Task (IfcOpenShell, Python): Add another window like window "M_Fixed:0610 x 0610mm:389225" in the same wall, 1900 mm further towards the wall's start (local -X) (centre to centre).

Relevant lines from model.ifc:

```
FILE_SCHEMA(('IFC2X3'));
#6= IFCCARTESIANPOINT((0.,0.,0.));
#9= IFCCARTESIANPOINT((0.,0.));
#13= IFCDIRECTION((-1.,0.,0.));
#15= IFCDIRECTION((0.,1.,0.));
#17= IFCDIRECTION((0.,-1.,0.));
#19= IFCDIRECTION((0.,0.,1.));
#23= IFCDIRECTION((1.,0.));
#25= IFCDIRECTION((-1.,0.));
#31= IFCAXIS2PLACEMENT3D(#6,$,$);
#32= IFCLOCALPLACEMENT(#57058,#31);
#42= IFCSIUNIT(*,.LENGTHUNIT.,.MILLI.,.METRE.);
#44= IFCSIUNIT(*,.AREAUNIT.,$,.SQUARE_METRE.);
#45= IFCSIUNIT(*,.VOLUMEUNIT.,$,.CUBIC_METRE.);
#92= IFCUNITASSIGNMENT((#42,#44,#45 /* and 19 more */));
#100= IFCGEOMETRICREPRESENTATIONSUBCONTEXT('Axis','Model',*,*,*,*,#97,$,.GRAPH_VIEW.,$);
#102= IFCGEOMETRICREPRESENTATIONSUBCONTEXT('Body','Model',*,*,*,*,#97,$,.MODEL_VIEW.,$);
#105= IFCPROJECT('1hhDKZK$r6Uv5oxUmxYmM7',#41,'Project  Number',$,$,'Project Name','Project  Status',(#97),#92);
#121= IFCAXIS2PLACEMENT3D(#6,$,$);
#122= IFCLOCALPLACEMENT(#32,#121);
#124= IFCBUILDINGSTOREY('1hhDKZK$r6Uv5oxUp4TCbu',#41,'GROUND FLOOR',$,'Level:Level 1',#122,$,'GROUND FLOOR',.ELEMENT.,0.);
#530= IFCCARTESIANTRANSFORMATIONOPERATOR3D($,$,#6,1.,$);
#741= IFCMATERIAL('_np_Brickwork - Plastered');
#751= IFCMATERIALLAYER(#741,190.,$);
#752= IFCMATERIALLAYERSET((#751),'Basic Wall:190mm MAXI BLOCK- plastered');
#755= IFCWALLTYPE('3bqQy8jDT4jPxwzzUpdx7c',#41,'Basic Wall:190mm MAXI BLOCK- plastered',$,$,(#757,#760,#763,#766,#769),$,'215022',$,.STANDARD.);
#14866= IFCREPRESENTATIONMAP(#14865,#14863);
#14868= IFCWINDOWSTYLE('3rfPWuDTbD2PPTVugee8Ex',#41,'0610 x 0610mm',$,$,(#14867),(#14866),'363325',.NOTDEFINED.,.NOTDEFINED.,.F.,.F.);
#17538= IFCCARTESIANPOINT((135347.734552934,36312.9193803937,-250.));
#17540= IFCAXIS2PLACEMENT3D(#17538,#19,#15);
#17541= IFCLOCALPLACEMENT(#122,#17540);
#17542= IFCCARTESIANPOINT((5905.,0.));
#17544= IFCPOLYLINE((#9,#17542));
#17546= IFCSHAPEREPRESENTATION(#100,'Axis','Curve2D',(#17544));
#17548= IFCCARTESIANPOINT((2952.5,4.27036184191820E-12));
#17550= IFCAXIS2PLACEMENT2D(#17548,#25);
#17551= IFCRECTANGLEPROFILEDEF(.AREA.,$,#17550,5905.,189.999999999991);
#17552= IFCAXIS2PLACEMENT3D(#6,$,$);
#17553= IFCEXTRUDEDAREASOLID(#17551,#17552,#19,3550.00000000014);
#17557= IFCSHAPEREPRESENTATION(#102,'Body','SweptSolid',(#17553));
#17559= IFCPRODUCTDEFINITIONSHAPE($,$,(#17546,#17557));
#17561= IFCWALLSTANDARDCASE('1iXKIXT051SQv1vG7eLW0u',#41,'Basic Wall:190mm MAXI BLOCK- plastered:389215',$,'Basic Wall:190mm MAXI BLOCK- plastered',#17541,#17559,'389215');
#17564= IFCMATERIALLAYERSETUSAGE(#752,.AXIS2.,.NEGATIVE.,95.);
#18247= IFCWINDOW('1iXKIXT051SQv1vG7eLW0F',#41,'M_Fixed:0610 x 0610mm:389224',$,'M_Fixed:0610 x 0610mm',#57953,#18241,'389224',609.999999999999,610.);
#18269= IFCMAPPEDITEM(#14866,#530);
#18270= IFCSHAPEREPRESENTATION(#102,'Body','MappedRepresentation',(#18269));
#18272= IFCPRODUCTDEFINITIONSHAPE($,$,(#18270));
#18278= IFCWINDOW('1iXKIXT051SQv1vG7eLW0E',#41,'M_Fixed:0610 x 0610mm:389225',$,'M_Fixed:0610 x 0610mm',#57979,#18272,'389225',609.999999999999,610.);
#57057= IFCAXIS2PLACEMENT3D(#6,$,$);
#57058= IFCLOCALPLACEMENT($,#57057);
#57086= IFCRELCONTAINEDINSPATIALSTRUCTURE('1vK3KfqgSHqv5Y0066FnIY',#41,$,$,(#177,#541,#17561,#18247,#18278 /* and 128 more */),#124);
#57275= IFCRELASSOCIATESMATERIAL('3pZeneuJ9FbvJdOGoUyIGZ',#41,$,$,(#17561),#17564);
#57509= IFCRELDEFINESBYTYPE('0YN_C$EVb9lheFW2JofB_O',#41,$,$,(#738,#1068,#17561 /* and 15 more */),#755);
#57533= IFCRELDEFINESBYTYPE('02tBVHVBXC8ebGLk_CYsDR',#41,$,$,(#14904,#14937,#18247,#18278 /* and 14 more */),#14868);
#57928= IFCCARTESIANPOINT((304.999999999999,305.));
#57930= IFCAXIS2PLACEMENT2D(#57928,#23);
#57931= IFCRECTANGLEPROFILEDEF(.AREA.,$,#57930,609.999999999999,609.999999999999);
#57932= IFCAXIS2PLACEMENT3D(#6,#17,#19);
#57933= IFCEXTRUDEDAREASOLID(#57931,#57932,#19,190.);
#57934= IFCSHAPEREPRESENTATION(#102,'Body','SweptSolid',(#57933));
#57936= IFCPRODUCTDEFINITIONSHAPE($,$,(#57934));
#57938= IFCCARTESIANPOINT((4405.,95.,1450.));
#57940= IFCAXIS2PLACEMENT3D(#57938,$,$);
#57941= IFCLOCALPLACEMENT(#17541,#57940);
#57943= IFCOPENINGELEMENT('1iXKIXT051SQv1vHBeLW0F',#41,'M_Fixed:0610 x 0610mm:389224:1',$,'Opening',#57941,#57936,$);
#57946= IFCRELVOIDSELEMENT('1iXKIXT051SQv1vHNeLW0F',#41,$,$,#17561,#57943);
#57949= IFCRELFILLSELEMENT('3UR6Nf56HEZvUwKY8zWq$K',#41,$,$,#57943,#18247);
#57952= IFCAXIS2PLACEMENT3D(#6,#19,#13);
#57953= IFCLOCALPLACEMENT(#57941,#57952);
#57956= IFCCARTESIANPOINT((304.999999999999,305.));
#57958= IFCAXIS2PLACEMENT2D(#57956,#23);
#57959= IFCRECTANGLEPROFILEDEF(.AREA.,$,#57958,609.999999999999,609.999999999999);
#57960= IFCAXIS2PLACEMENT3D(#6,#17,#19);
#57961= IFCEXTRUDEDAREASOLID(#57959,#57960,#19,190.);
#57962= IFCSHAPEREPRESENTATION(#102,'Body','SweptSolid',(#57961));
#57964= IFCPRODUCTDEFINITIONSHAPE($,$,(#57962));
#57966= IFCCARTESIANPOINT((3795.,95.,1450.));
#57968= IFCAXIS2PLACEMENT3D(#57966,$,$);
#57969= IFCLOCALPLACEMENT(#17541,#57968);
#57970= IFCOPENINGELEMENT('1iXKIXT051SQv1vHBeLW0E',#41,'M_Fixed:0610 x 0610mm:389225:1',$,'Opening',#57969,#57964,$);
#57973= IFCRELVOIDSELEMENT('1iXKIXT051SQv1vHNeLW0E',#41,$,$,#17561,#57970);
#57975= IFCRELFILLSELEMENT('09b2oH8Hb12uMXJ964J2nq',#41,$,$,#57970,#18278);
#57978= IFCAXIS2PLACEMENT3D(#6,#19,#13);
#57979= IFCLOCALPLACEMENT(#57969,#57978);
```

```python
import ifcopenshell
import ifcopenshell.api.feature
import ifcopenshell.api.geometry
import ifcopenshell.api.root
import ifcopenshell.geom
import ifcopenshell.util.element
import ifcopenshell.util.placement
import ifcopenshell.util.shape

model = ifcopenshell.open("model.ifc")
settings = ifcopenshell.geom.settings()


def volume(element):
    """Net volume in cubic metres, openings subtracted."""
    shape = ifcopenshell.geom.create_shape(settings, element)
    return ifcopenshell.util.shape.get_volume(shape.geometry)


def reuse_history(source, copy):
    """copy_class also copies each property set's owner history, people and application; keep the originals."""
    for rel in copy.IsDefinedBy:
        if rel.is_a("IfcRelDefinesByProperties") and (history := rel.RelatingPropertyDefinition.OwnerHistory):
            rel.RelatingPropertyDefinition.OwnerHistory = source.OwnerHistory
            ifcopenshell.util.element.remove_deep2(model, history)


window = model.by_guid("1iXKIXT051SQv1vG7eLW0E")
opening = window.FillsVoids[0].RelatingOpeningElement
wall = opening.VoidsElements[0].RelatingBuildingElement
before = volume(wall)
shift = ifcopenshell.util.placement.get_local_placement(wall.ObjectPlacement)[:3, 0] * -1900.0

# copy_class copies the void relationship, type, container and properties, but no geometry.
new_opening = ifcopenshell.api.root.copy_class(model, product=opening)
new_opening.Representation = ifcopenshell.util.element.copy_deep(
    model, opening.Representation, exclude=["IfcGeometricRepresentationContext", "IfcRepresentationMap"]
)
new_opening.Name = "M_Fixed:0610 x 0610mm"
new_window = ifcopenshell.api.root.copy_class(model, product=window)
new_window.Representation = ifcopenshell.util.element.copy_deep(
    model, window.Representation, exclude=["IfcGeometricRepresentationContext", "IfcRepresentationMap"]
)
new_window.Name = "M_Fixed:0610 x 0610mm"
new_window.Tag = None
reuse_history(window, new_window)
fills = ifcopenshell.api.feature.add_filling(model, opening=new_opening, element=new_window)
fills.OwnerHistory = new_window.OwnerHistory  # required in IFC2X3

for old, new in ((opening, new_opening), (window, new_window)):
    matrix = ifcopenshell.util.placement.get_local_placement(old.ObjectPlacement)
    matrix[:3, 3] += shift
    ifcopenshell.api.geometry.edit_object_placement(model, product=new, matrix=matrix, is_si=False)

after = volume(wall)

print(f"wall volume {before:.3f} -> {after:.3f} m3")

model.write("model_edited.ifc")
```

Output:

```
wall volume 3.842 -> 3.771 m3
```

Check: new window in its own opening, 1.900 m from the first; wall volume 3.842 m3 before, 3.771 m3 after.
